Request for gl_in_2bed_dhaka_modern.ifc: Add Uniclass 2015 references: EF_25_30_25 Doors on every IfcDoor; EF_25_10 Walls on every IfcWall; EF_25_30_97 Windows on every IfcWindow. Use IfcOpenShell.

First a look at what the model holds.

```python
import ifcopenshell

model = ifcopenshell.open("gl_in_2bed_dhaka_modern.ifc")
print(model.schema)
print("classifications:", [c.Name for c in model.by_type("IfcClassification")])
for ifc_class in ("IfcDoor", "IfcRoof", "IfcStair", "IfcWall", "IfcWindow"):
    print(ifc_class, len(model.by_type(ifc_class)))
```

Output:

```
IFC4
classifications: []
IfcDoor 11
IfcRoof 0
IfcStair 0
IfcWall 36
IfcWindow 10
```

```python
import ifcopenshell
import ifcopenshell.api.classification

model = ifcopenshell.open("gl_in_2bed_dhaka_modern.ifc")

system = ifcopenshell.api.classification.add_classification(model, classification="Uniclass 2015")

codes = {
    "IfcDoor": ("EF_25_30_25", "Doors"),
    "IfcWall": ("EF_25_10", "Walls"),
    "IfcWindow": ("EF_25_30_97", "Windows"),
}
for ifc_class, (code, name) in codes.items():
    products = model.by_type(ifc_class)
    ifcopenshell.api.classification.add_reference(
        model, products=products, classification=system, identification=code, name=name
    )
    print(code, len(products))

model.write("gl_in_2bed_dhaka_modern-out.ifc")
```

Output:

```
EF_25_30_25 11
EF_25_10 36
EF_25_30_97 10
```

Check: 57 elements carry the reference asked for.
